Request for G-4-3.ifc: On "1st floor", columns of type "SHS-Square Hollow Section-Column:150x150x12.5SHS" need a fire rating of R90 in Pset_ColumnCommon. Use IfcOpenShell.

First a look at what the model holds.

```python
import ifcopenshell
import ifcopenshell.util.element

model = ifcopenshell.open("G-4-3.ifc")
print(model.schema)
storey = next(s for s in model.by_type("IfcBuildingStorey") if s.Name == "1st floor")
columns = [e for e in ifcopenshell.util.element.get_decomposition(storey) if e.is_a("IfcColumn")]
seen = {}
for e in columns:
    element_type = ifcopenshell.util.element.get_type(e)
    key = (element_type.Name if element_type != e and element_type else None, ifcopenshell.util.element.get_pset(e, "Pset_ColumnCommon", "FireRating"))
    seen[key] = seen.get(key, 0) + 1
for (name, value), count in sorted(seen.items(), key=str):
    print(count, "x", name, "|", value)
```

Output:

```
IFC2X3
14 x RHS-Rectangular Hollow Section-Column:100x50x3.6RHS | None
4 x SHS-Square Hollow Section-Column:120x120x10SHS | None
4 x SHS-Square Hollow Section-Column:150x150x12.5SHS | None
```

```python
import ifcopenshell
import ifcopenshell.api.pset
import ifcopenshell.util.element

model = ifcopenshell.open("G-4-3.ifc")

storey = next(s for s in model.by_type("IfcBuildingStorey") if s.Name == "1st floor")
columns = [e for e in ifcopenshell.util.element.get_decomposition(storey) if e.is_a("IfcColumn")]

count = 0
for e in columns:
    element_type = ifcopenshell.util.element.get_type(e)
    if element_type in (None, e) or element_type.Name != "SHS-Square Hollow Section-Column:150x150x12.5SHS":
        continue
    # add_pset returns the element's existing set when there is one.
    pset = ifcopenshell.api.pset.add_pset(model, product=e, name="Pset_ColumnCommon")
    ifcopenshell.api.pset.edit_pset(model, pset=pset, properties={"FireRating": "R90"})
    count += 1

print(count, "columns updated")

model.write("G-4-3_edited.ifc")
```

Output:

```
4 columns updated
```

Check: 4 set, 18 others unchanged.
